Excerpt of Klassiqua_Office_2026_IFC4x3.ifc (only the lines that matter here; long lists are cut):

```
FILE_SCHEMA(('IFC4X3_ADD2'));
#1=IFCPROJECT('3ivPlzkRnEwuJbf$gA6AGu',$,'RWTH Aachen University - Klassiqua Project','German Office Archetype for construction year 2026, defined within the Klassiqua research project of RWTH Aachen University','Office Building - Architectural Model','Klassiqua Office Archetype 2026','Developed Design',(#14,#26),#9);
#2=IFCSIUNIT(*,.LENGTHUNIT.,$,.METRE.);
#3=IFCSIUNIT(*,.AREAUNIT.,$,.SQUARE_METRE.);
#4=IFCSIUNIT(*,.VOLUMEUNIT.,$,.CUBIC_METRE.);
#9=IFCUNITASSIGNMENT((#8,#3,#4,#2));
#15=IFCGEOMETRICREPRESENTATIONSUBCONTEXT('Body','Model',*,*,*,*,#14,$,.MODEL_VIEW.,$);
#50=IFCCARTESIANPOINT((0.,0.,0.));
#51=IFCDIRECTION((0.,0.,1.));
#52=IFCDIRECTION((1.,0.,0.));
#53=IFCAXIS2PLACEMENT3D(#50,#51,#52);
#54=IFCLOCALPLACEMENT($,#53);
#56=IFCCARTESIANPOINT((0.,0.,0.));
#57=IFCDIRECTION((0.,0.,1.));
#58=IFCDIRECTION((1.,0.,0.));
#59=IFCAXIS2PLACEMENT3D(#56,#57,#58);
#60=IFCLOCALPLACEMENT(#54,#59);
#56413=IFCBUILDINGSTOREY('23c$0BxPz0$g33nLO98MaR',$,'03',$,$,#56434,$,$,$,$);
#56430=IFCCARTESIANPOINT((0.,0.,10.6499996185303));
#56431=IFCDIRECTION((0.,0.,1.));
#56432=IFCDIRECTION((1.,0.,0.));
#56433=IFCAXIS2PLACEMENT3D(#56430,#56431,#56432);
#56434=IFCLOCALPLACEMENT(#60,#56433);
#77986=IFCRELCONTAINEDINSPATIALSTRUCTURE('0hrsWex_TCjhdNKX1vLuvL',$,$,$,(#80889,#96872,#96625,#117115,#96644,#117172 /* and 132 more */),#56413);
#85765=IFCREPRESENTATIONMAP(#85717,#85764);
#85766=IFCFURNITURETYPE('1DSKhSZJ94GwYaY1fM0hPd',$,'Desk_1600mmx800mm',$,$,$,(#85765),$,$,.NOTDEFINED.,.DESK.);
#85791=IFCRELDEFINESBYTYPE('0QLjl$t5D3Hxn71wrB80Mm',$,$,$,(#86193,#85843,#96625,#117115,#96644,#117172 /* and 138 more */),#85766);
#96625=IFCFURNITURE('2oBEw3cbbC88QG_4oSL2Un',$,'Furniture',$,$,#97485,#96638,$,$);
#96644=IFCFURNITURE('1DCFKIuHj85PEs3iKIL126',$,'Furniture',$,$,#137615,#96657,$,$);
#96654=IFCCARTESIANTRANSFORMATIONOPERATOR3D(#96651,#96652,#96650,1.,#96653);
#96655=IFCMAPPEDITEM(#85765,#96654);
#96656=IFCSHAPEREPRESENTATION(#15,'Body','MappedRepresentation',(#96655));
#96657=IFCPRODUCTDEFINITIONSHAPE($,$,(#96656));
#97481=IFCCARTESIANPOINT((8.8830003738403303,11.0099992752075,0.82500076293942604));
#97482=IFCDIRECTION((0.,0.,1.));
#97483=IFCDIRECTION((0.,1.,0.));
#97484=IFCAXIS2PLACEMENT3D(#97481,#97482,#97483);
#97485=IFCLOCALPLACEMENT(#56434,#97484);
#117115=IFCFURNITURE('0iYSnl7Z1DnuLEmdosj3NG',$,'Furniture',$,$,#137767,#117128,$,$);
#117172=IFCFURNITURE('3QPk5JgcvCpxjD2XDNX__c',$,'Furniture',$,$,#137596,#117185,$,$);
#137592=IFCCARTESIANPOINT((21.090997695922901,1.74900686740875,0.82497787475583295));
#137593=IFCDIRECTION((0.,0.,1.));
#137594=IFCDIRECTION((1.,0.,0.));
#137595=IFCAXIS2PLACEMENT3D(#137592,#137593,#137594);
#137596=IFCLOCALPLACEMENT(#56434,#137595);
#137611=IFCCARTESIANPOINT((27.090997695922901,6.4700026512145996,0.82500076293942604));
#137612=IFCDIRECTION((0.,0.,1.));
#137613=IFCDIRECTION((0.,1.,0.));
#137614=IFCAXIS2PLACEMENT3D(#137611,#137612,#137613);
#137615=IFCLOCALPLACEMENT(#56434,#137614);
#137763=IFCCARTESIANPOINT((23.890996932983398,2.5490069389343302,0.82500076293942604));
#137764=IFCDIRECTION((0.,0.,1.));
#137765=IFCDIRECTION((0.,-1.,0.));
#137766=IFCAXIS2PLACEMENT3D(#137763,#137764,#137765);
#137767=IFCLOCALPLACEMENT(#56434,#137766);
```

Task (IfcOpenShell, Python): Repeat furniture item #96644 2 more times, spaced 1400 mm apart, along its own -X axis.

```python
import ifcopenshell
import ifcopenshell.api.geometry
import ifcopenshell.api.root
import ifcopenshell.util.element
import ifcopenshell.util.placement
import ifcopenshell.util.unit

model = ifcopenshell.open("Klassiqua_Office_2026_IFC4x3.ifc")
unit_scale = ifcopenshell.util.unit.calculate_unit_scale(model)

source = model.by_guid("1DCFKIuHj85PEs3iKIL126")
base = ifcopenshell.util.placement.get_local_placement(source.ObjectPlacement)
step = -base[:3, 0] * 1.4 / unit_scale

for i in range(1, 3):
    copy = ifcopenshell.api.root.copy_class(model, product=source)
    copy.Representation = ifcopenshell.util.element.copy_deep(
        model, source.Representation, exclude=["IfcGeometricRepresentationContext", "IfcRepresentationMap"]
    )
    matrix = base.copy()
    matrix[:3, 3] += i * step
    print("added at", matrix[:3, 3].round(3) + 0.0)
    ifcopenshell.api.geometry.edit_object_placement(model, product=copy, matrix=matrix, is_si=False)

model.write("Klassiqua_Office_2026_IFC4x3_v2.ifc")
```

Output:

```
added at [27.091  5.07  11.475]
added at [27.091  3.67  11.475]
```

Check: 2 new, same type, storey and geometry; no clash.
